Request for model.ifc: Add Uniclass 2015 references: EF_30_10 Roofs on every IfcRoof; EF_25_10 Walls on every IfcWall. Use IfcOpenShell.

First a look at what the model holds.

```python
import ifcopenshell

model = ifcopenshell.open("model.ifc")
print(model.schema)
print("classifications:", [c.Name for c in model.by_type("IfcClassification")])
for ifc_class in ("IfcDoor", "IfcRoof", "IfcStair", "IfcWall", "IfcWindow"):
    print(ifc_class, len(model.by_type(ifc_class)))
```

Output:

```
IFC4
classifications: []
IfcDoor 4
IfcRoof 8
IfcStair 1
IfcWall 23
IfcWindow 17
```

```python
import ifcopenshell
import ifcopenshell.api.classification

model = ifcopenshell.open("model.ifc")

system = ifcopenshell.api.classification.add_classification(model, classification="Uniclass 2015")

codes = {
    "IfcRoof": ("EF_30_10", "Roofs"),
    "IfcWall": ("EF_25_10", "Walls"),
}
for ifc_class, (code, name) in codes.items():
    products = model.by_type(ifc_class)
    ifcopenshell.api.classification.add_reference(
        model, products=products, classification=system, identification=code, name=name
    )
    print(code, len(products))

model.write("model_updated.ifc")
```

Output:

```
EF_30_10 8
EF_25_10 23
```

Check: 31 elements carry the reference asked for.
